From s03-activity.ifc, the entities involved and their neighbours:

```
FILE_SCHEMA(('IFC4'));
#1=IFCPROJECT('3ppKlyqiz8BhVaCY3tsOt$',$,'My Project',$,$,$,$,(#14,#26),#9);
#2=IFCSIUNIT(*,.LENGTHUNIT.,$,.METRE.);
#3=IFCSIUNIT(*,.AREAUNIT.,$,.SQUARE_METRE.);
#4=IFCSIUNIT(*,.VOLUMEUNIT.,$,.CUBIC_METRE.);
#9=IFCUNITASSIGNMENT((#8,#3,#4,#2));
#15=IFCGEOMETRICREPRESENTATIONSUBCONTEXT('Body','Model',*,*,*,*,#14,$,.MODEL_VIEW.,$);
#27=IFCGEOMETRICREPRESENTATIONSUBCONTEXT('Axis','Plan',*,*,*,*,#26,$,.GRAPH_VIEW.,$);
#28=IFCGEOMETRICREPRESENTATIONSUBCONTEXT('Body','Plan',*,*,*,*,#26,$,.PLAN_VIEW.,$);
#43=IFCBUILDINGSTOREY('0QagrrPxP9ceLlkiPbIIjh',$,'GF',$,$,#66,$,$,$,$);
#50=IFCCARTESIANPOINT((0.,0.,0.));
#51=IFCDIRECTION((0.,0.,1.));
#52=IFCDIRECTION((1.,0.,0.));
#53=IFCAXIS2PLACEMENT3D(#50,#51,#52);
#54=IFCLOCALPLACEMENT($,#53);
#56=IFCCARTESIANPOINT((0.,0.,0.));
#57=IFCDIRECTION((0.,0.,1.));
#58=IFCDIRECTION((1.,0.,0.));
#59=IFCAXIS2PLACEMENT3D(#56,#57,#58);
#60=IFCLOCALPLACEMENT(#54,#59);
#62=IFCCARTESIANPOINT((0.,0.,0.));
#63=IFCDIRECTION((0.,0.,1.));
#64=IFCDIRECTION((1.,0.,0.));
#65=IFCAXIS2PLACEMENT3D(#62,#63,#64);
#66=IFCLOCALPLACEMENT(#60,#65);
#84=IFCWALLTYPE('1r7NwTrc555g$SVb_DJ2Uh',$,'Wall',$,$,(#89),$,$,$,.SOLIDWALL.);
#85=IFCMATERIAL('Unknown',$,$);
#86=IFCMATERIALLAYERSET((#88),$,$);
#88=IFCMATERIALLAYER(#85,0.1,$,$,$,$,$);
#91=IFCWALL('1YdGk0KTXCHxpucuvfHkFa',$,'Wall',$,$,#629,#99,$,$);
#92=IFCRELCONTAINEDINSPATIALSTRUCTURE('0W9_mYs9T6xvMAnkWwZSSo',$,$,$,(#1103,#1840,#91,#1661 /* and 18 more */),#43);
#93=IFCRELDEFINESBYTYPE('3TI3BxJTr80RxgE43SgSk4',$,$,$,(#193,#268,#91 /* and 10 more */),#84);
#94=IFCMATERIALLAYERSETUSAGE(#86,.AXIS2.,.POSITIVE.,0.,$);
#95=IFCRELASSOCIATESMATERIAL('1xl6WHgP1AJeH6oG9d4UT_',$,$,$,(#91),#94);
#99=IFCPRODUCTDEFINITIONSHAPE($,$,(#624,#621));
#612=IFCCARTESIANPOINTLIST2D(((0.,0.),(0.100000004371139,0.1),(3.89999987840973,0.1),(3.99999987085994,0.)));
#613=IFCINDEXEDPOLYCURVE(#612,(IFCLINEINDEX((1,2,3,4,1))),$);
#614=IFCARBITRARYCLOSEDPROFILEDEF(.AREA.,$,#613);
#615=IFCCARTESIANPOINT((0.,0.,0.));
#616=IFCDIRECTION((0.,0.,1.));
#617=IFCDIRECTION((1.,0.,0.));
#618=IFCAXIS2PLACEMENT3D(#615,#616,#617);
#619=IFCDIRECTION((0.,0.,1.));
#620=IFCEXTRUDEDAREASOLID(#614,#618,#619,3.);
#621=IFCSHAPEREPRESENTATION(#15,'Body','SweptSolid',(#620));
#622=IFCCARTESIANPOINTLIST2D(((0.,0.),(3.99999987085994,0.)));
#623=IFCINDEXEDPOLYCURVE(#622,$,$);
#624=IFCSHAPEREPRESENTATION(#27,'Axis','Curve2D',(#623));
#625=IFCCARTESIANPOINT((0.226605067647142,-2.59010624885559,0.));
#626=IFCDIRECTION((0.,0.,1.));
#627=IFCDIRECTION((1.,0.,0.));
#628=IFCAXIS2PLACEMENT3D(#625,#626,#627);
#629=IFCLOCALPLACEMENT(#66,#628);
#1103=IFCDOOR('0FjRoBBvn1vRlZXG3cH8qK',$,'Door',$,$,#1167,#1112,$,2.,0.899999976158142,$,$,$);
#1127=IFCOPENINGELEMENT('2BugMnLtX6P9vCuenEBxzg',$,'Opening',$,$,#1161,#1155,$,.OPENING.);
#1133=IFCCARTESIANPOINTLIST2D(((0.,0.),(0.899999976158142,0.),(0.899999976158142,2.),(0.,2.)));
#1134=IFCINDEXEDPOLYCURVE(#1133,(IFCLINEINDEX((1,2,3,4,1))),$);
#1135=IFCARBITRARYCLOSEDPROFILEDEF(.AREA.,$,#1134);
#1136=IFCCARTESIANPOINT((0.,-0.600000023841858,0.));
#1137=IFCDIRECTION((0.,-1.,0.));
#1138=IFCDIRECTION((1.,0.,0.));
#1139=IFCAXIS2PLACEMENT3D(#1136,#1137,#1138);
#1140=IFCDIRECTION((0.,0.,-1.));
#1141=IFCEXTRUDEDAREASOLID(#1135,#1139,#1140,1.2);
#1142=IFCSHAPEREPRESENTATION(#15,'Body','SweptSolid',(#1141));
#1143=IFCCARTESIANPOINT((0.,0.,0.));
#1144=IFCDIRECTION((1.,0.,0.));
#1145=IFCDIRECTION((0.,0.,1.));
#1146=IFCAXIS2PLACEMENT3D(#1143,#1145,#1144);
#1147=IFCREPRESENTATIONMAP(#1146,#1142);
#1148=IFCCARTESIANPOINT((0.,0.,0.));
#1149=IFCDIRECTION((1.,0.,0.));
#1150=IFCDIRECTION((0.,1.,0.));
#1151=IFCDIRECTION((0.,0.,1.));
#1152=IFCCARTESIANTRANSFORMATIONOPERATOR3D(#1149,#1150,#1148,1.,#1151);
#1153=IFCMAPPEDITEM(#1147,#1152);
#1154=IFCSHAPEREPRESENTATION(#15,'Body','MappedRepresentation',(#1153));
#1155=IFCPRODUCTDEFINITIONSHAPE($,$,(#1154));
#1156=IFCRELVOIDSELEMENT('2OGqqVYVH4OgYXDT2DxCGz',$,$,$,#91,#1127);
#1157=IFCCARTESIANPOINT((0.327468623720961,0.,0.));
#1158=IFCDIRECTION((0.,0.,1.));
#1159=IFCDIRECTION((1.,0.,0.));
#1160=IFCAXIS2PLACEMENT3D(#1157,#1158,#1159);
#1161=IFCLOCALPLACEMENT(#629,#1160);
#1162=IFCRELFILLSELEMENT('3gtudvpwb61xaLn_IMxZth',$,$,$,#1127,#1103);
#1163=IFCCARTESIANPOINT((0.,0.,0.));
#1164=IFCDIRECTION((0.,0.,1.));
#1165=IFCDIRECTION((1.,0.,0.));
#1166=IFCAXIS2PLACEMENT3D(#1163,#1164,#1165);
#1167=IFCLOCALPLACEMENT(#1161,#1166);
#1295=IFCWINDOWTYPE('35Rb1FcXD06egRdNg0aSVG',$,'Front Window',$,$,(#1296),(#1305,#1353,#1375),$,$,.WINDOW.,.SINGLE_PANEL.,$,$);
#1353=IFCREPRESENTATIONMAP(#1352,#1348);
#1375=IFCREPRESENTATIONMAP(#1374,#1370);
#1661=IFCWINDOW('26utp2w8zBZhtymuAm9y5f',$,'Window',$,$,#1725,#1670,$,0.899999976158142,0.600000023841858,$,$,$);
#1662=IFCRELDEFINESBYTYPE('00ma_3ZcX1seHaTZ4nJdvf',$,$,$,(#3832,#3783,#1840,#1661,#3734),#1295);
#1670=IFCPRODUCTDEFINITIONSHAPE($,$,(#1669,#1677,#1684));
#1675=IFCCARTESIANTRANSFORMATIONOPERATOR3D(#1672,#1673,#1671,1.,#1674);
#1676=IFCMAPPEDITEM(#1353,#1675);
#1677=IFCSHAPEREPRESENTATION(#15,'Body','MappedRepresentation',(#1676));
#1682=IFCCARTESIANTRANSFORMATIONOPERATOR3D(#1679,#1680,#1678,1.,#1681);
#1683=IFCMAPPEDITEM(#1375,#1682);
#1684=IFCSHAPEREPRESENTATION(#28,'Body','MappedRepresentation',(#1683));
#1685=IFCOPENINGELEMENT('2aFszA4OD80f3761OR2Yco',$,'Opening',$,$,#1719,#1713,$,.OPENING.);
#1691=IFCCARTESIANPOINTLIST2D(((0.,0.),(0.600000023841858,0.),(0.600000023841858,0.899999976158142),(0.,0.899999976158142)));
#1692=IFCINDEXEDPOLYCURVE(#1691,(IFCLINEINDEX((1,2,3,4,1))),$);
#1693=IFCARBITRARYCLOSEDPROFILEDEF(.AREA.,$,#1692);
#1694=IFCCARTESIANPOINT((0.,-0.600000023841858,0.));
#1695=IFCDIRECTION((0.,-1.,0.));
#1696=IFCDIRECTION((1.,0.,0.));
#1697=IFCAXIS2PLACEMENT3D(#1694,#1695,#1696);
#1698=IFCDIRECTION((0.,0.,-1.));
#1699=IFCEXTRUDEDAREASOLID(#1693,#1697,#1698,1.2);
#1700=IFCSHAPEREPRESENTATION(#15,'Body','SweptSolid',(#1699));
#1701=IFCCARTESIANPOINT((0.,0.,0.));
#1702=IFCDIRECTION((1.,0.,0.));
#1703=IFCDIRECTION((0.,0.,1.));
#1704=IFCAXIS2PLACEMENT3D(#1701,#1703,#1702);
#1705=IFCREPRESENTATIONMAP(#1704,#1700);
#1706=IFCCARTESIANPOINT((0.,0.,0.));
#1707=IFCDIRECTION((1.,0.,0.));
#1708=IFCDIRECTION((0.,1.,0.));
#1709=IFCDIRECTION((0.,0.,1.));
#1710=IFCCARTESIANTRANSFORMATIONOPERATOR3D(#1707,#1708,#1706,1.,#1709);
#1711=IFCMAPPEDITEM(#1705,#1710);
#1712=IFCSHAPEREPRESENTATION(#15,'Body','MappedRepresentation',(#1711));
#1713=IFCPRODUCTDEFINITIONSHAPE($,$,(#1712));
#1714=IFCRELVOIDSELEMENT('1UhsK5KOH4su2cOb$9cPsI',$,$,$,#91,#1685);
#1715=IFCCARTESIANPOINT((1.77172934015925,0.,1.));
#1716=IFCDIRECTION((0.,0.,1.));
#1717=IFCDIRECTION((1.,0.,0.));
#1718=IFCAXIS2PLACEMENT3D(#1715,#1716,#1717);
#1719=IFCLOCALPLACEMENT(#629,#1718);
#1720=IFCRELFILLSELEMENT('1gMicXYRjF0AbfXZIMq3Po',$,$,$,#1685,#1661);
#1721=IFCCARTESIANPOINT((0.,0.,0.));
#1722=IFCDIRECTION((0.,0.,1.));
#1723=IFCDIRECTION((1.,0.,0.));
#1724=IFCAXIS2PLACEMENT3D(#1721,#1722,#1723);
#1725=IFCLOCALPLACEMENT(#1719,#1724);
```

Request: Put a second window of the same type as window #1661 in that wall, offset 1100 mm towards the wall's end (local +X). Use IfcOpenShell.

```python
import ifcopenshell
import ifcopenshell.api.feature
import ifcopenshell.api.geometry
import ifcopenshell.api.root
import ifcopenshell.geom
import ifcopenshell.util.element
import ifcopenshell.util.placement
import ifcopenshell.util.shape
import ifcopenshell.util.unit

model = ifcopenshell.open("s03-activity.ifc")
unit_scale = ifcopenshell.util.unit.calculate_unit_scale(model)
settings = ifcopenshell.geom.settings()


def volume(element):
    """Net volume in cubic metres, openings subtracted."""
    shape = ifcopenshell.geom.create_shape(settings, element)
    return ifcopenshell.util.shape.get_volume(shape.geometry)


window = model.by_guid("26utp2w8zBZhtymuAm9y5f")
opening = window.FillsVoids[0].RelatingOpeningElement
wall = opening.VoidsElements[0].RelatingBuildingElement
before = volume(wall)
shift = ifcopenshell.util.placement.get_local_placement(wall.ObjectPlacement)[:3, 0] * 1.1 / unit_scale

# copy_class copies the void relationship, type, container and properties, but no geometry.
new_opening = ifcopenshell.api.root.copy_class(model, product=opening)
new_opening.Representation = ifcopenshell.util.element.copy_deep(
    model, opening.Representation, exclude=["IfcGeometricRepresentationContext", "IfcRepresentationMap"]
)
new_window = ifcopenshell.api.root.copy_class(model, product=window)
new_window.Representation = ifcopenshell.util.element.copy_deep(
    model, window.Representation, exclude=["IfcGeometricRepresentationContext", "IfcRepresentationMap"]
)
ifcopenshell.api.feature.add_filling(model, opening=new_opening, element=new_window)

for old, new in ((opening, new_opening), (window, new_window)):
    matrix = ifcopenshell.util.placement.get_local_placement(old.ObjectPlacement)
    matrix[:3, 3] += shift
    ifcopenshell.api.geometry.edit_object_placement(model, product=new, matrix=matrix, is_si=False)

after = volume(wall)

print(f"wall volume {before:.3f} -> {after:.3f} m3")

model.write("s03-activity_updated.ifc")
```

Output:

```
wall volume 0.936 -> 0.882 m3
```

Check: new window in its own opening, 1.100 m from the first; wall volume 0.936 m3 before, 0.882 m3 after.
